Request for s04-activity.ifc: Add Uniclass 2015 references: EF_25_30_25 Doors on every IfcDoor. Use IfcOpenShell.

First a look at what the model holds.

```python
import ifcopenshell

model = ifcopenshell.open("s04-activity.ifc")
print(model.schema)
print("classifications:", [c.Name for c in model.by_type("IfcClassification")])
for ifc_class in ("IfcDoor", "IfcRoof", "IfcStair", "IfcWall", "IfcWindow"):
    print(ifc_class, len(model.by_type(ifc_class)))
```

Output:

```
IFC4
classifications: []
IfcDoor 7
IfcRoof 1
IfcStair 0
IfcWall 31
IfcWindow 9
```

```python
import ifcopenshell
import ifcopenshell.api.classification

model = ifcopenshell.open("s04-activity.ifc")

system = ifcopenshell.api.classification.add_classification(model, classification="Uniclass 2015")

codes = {
    "IfcDoor": ("EF_25_30_25", "Doors"),
}
for ifc_class, (code, name) in codes.items():
    products = model.by_type(ifc_class)
    ifcopenshell.api.classification.add_reference(
        model, products=products, classification=system, identification=code, name=name
    )
    print(code, len(products))

model.write("s04-activity_v2.ifc")
```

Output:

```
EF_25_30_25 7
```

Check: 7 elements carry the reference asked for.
